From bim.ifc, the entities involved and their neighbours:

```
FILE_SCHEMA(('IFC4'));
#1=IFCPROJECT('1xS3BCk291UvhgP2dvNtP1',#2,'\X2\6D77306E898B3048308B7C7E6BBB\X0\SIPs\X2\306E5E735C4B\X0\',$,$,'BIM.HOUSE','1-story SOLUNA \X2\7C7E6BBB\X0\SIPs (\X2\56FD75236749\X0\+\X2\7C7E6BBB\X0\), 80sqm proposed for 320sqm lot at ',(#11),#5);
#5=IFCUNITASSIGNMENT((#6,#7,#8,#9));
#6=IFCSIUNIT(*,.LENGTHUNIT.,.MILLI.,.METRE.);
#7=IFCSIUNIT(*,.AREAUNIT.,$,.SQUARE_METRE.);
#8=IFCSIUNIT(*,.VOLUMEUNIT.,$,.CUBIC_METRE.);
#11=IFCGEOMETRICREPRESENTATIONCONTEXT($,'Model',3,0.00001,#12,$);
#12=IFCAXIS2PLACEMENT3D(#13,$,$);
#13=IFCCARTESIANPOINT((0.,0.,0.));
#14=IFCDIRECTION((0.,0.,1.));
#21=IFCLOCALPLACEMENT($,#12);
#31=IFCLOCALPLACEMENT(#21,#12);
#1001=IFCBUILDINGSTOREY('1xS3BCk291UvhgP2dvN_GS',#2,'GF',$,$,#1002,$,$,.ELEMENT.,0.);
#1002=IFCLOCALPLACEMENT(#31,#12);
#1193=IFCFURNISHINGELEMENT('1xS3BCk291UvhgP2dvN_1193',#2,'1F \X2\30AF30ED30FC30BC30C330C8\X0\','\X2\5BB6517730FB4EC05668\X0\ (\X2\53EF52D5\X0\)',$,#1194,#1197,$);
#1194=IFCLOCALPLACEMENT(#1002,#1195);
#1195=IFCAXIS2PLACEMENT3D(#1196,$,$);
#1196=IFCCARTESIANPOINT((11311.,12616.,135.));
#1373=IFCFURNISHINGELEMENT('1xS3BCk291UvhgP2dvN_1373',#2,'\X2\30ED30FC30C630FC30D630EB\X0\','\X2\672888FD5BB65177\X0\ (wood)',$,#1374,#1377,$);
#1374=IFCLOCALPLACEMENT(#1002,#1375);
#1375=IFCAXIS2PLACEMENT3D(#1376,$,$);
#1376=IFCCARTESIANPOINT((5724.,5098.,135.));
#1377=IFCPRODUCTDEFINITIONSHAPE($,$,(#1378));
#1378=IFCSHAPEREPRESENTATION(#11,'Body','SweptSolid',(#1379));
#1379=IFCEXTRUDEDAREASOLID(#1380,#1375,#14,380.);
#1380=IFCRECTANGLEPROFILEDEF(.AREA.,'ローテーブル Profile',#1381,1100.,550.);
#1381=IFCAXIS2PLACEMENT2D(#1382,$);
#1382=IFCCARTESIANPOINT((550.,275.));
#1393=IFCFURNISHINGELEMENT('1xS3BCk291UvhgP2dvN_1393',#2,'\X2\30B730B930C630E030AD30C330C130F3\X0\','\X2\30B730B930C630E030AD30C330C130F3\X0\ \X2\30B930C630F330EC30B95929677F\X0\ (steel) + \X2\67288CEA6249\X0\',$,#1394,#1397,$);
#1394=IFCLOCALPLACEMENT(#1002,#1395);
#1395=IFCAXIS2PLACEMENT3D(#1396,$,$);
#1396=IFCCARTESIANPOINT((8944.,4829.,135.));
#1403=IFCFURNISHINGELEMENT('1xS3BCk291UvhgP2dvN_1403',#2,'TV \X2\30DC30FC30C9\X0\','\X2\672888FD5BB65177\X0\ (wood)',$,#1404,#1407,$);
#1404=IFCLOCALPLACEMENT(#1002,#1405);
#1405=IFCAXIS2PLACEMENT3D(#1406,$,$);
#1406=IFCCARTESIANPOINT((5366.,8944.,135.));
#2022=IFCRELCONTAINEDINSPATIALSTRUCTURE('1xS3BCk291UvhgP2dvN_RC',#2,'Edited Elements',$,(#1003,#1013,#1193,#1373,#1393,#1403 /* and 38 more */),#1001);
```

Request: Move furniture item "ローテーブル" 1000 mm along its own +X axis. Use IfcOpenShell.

```python
import ifcopenshell
import ifcopenshell.api.geometry
import ifcopenshell.util.placement
import ifcopenshell.util.unit

model = ifcopenshell.open("bim.ifc")
unit_scale = ifcopenshell.util.unit.calculate_unit_scale(model)

item = model.by_id(1373)
matrix = ifcopenshell.util.placement.get_local_placement(item.ObjectPlacement)
matrix[:3, 3] += matrix[:3, 0] * 1 / unit_scale
ifcopenshell.api.geometry.edit_object_placement(model, product=item, matrix=matrix, is_si=False)

print(ifcopenshell.util.placement.get_local_placement(item.ObjectPlacement).round(3) + 0.0)

model.write("bim_rev.ifc")
```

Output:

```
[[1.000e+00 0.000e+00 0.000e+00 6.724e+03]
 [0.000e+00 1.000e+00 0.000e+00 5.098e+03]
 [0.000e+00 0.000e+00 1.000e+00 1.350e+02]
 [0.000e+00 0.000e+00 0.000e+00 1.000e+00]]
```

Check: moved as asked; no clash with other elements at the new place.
